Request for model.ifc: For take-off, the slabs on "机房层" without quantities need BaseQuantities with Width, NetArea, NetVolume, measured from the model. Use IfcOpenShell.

First a look at what the model holds.

```python
import ifcopenshell
import ifcopenshell.util.element
import ifcopenshell.util.unit

model = ifcopenshell.open("model.ifc")
print(model.schema)
for unit_type in ("LENGTHUNIT", "AREAUNIT", "VOLUMEUNIT"):
    print(unit_type, ifcopenshell.util.unit.calculate_unit_scale(model, unit_type))
storey = next(s for s in model.by_type("IfcBuildingStorey") if s.Name == "机房层")
slabs = [e for e in ifcopenshell.util.element.get_decomposition(storey) if e.is_a("IfcSlab")]
for e in sorted(slabs, key=lambda e: e.id()):
    print(e.id(), e.is_a(), e.Name, list(ifcopenshell.util.element.get_psets(e, qtos_only=True)), sep=" | ")
```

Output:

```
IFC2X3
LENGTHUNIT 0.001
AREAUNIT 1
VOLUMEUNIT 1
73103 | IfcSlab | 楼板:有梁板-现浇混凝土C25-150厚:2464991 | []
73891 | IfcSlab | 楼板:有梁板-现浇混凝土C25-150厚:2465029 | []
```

```python
import ifcopenshell
import ifcopenshell.api.pset
import ifcopenshell.geom
import ifcopenshell.util.element
import ifcopenshell.util.shape
import ifcopenshell.util.unit

model = ifcopenshell.open("model.ifc")
unit_scale = ifcopenshell.util.unit.calculate_unit_scale(model)
area_scale = ifcopenshell.util.unit.calculate_unit_scale(model, "AREAUNIT")
volume_scale = ifcopenshell.util.unit.calculate_unit_scale(model, "VOLUMEUNIT")
settings = ifcopenshell.geom.settings()

storey = next(s for s in model.by_type("IfcBuildingStorey") if s.Name == "机房层")
slabs = [e for e in ifcopenshell.util.element.get_decomposition(storey) if e.is_a("IfcSlab")]

for e in sorted(slabs, key=lambda e: e.id()):
    if ifcopenshell.util.element.get_psets(e, qtos_only=True, should_inherit=False):
        continue
    # Geometry comes back in metres, in the element's own axes.
    shape = ifcopenshell.geom.create_shape(settings, e)
    values = {
        "Width": ifcopenshell.util.shape.get_z(shape.geometry) / unit_scale,
        "NetArea": ifcopenshell.util.shape.get_footprint_area(shape.geometry) / area_scale,
        "NetVolume": ifcopenshell.util.shape.get_volume(shape.geometry) / volume_scale,
    }
    qto = ifcopenshell.api.pset.add_qto(model, product=e, name="BaseQuantities")
    ifcopenshell.api.pset.edit_qto(model, qto=qto, properties=values)
    print(e.id(), {k: round(v, 3) for k, v in values.items()})

model.write("model_updated.ifc")
```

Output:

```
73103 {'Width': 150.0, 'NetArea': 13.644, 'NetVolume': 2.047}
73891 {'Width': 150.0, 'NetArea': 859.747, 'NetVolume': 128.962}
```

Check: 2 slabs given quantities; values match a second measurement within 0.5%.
